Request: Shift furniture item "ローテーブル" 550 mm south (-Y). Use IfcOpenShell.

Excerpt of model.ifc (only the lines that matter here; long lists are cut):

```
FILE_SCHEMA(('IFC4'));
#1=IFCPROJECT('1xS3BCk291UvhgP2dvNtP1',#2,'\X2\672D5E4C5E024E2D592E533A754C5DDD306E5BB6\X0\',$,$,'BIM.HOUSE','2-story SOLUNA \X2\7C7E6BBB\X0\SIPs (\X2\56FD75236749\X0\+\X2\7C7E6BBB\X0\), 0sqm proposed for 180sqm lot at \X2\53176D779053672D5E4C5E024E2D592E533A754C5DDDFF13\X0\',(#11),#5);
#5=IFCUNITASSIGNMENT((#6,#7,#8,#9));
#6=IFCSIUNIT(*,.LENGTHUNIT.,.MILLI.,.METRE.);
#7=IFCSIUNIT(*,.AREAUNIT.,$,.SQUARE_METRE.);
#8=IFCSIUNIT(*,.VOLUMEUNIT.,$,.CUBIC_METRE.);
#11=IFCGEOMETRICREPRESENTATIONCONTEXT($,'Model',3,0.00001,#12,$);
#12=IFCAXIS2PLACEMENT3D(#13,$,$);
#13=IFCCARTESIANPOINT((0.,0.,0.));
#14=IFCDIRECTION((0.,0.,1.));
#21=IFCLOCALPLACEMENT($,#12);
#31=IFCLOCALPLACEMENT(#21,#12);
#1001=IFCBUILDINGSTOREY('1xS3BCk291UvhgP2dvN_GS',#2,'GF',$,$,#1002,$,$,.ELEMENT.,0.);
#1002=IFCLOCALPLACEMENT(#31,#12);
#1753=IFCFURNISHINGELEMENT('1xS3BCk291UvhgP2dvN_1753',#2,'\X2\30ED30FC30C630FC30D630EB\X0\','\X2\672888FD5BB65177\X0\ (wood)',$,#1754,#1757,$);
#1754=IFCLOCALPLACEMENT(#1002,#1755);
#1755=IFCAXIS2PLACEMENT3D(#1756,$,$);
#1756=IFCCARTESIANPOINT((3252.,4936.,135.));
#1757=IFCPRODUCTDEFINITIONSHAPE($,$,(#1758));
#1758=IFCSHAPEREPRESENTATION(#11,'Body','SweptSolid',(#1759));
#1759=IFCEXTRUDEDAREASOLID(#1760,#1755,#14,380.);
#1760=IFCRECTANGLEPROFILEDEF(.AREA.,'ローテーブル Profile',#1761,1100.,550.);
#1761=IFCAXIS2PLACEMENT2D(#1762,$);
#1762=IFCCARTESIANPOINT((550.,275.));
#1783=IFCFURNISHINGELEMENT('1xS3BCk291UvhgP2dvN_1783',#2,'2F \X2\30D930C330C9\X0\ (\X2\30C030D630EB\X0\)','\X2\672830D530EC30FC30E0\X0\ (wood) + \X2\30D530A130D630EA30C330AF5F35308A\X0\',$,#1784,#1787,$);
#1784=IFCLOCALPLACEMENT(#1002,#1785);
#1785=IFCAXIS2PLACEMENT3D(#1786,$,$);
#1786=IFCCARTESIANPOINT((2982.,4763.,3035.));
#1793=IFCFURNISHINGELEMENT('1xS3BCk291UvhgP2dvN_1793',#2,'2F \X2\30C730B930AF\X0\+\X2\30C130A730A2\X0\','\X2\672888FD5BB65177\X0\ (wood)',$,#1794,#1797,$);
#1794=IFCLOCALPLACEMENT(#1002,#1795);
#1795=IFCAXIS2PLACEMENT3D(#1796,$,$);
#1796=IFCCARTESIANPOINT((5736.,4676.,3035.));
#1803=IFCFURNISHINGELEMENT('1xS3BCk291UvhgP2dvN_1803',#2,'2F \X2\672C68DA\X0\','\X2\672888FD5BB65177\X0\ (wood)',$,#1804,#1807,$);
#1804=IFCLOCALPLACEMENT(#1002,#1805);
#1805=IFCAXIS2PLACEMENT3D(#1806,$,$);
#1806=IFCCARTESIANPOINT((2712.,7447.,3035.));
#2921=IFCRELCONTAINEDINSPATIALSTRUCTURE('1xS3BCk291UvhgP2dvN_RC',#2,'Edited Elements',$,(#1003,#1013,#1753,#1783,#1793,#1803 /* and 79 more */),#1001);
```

```python
import ifcopenshell
import ifcopenshell.api.geometry
import ifcopenshell.util.placement
import ifcopenshell.util.unit

model = ifcopenshell.open("model.ifc")
unit_scale = ifcopenshell.util.unit.calculate_unit_scale(model)

item = model.by_id(1753)
matrix = ifcopenshell.util.placement.get_local_placement(item.ObjectPlacement)
matrix[1, 3] -= 0.55 / unit_scale
ifcopenshell.api.geometry.edit_object_placement(model, product=item, matrix=matrix, is_si=False)

print(ifcopenshell.util.placement.get_local_placement(item.ObjectPlacement).round(3) + 0.0)

model.write("model_rev.ifc")
```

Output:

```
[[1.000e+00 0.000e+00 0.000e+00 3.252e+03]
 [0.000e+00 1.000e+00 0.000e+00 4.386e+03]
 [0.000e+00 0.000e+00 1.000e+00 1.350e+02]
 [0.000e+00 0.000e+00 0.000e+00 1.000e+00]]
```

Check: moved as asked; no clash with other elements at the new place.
